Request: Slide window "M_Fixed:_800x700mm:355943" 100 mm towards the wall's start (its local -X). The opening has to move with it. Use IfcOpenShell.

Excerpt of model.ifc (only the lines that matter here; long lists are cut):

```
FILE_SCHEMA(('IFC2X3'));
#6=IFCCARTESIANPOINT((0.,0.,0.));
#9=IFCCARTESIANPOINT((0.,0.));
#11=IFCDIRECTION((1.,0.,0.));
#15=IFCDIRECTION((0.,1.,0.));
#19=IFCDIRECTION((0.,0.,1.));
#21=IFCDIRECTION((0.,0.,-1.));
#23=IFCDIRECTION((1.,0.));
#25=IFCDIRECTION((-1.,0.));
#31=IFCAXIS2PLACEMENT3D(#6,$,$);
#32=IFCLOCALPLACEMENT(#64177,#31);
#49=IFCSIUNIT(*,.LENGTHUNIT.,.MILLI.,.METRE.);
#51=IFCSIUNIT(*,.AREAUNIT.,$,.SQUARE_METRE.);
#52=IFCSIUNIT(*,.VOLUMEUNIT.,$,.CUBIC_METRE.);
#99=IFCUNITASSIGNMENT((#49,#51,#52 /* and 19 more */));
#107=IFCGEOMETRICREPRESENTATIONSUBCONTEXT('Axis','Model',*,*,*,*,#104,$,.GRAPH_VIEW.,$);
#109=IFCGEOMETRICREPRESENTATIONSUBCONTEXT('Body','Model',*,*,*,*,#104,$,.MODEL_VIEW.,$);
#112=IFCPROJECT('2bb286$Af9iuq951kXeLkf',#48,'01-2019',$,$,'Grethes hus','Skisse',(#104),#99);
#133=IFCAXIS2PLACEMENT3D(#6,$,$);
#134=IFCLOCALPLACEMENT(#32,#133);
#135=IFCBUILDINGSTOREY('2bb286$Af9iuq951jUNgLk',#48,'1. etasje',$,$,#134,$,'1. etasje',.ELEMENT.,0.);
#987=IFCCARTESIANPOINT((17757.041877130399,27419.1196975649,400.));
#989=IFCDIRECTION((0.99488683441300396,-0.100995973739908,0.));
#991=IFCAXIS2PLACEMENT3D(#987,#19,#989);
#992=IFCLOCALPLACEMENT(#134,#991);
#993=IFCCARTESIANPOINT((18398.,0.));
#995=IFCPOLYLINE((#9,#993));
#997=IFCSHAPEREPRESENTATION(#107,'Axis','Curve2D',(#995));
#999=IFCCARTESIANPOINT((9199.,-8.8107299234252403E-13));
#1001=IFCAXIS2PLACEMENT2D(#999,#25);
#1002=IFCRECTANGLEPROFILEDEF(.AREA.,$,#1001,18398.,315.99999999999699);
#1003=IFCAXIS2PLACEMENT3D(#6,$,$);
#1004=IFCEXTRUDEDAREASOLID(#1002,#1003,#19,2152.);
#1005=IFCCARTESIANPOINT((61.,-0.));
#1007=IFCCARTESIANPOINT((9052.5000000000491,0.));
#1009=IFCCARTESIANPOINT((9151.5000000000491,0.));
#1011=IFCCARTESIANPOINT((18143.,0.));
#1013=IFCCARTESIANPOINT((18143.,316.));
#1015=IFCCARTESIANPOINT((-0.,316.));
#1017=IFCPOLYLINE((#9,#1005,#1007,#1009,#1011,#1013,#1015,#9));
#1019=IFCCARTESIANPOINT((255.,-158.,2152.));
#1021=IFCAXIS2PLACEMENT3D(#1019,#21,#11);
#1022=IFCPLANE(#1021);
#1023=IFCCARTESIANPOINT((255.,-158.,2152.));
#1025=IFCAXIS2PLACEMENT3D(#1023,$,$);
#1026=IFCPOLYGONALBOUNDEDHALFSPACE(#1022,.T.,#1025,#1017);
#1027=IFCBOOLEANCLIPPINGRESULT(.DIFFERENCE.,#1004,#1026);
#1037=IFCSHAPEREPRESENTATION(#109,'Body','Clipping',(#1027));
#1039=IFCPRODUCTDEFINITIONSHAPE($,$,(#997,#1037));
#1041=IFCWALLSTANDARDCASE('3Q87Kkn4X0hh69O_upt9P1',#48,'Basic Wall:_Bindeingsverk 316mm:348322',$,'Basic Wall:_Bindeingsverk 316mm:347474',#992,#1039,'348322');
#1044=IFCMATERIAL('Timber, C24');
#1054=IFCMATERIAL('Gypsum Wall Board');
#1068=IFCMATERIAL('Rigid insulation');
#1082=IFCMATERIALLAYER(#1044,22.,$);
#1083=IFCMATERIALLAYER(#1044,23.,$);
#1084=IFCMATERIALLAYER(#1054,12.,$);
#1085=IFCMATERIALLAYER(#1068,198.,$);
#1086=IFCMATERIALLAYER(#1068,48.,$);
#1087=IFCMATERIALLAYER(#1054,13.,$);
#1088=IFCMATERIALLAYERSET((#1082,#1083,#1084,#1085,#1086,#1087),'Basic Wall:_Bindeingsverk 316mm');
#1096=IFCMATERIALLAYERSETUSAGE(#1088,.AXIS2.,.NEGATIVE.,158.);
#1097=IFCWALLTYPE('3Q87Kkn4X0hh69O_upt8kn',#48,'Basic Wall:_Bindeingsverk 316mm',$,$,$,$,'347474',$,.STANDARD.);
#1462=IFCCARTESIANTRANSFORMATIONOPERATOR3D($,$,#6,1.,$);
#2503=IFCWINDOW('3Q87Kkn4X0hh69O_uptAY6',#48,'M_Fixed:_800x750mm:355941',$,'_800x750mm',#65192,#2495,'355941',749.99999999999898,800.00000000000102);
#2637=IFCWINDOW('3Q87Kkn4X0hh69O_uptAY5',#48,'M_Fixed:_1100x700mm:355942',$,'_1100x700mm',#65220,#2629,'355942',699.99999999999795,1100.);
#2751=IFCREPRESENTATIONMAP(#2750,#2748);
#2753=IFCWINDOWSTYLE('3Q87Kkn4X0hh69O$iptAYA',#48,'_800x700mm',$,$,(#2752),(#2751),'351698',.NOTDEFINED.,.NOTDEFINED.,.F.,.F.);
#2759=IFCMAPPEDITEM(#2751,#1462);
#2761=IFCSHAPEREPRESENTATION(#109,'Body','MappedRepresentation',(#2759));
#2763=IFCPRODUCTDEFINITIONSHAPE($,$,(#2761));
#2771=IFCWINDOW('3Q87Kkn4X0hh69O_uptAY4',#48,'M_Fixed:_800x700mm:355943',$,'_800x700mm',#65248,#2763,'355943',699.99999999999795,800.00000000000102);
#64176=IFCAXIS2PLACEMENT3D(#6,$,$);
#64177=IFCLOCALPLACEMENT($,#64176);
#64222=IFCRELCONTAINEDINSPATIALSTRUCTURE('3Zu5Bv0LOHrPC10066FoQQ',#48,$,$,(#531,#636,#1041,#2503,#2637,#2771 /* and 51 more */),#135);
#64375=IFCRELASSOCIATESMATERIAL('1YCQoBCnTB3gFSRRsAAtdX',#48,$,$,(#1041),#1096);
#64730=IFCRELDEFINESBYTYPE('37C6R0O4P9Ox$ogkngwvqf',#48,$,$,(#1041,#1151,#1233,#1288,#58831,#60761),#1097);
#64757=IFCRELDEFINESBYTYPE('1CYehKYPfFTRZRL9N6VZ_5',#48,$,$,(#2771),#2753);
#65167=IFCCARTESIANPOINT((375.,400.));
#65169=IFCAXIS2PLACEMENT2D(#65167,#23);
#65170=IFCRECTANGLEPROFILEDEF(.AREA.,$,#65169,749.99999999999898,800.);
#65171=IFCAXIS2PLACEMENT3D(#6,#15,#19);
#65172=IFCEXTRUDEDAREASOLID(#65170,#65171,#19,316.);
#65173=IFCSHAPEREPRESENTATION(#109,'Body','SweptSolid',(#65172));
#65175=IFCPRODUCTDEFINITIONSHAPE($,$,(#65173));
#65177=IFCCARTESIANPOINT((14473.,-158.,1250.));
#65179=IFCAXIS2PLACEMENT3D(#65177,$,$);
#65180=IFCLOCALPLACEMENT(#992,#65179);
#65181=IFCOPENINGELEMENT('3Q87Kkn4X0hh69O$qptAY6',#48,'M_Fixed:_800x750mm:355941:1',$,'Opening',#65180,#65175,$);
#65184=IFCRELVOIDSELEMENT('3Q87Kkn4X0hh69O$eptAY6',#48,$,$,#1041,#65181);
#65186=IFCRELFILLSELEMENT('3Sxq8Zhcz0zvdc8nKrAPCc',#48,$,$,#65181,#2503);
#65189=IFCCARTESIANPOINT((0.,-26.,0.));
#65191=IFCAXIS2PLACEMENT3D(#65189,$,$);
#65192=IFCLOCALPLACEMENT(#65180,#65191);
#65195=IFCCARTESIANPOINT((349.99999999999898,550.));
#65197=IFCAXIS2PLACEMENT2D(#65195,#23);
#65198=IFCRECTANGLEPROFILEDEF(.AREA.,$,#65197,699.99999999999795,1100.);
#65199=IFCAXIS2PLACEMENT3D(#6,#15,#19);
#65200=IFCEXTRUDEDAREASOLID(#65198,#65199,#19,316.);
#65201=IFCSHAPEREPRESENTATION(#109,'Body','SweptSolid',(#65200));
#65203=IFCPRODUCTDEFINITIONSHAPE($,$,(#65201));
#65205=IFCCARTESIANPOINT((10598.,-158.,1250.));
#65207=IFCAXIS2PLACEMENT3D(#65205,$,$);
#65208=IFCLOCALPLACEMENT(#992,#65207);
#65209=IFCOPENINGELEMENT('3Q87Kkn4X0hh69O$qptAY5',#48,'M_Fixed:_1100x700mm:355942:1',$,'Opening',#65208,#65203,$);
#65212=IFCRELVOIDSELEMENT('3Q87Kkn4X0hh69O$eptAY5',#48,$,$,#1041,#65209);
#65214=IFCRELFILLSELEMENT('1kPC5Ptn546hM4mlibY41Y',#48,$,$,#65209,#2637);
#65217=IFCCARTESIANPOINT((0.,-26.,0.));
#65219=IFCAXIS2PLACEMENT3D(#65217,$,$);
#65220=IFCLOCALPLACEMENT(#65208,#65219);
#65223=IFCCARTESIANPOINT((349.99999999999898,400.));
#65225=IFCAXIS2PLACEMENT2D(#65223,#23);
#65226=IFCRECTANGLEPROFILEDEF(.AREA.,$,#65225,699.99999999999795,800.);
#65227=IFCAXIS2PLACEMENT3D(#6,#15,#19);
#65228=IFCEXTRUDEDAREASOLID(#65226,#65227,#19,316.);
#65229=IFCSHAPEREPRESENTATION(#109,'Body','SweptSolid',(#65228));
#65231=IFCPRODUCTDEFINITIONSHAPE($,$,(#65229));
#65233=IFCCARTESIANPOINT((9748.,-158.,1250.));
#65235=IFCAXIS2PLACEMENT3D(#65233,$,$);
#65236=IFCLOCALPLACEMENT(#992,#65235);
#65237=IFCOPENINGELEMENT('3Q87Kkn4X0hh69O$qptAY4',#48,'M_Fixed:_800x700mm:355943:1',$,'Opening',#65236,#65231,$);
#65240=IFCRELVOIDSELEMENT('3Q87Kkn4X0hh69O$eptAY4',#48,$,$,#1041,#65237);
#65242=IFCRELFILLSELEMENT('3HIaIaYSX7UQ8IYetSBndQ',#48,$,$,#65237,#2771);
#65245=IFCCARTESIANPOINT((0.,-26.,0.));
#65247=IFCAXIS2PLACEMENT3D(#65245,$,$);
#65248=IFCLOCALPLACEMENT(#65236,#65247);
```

```python
import ifcopenshell
import ifcopenshell.api.geometry
import ifcopenshell.util.placement
import ifcopenshell.util.unit

model = ifcopenshell.open("model.ifc")
unit_scale = ifcopenshell.util.unit.calculate_unit_scale(model)

window = model.by_guid("3Q87Kkn4X0hh69O_uptAY4")
opening = window.FillsVoids[0].RelatingOpeningElement
wall = opening.VoidsElements[0].RelatingBuildingElement

wall_matrix = ifcopenshell.util.placement.get_local_placement(wall.ObjectPlacement)
shift = wall_matrix[:3, 0] * -0.1 / unit_scale
before = ifcopenshell.util.placement.get_local_placement(window.ObjectPlacement)[:3, 3].copy()

# The window is placed relative to its opening, so it follows when the opening moves.
matrix = ifcopenshell.util.placement.get_local_placement(opening.ObjectPlacement)
matrix[:3, 3] += shift
ifcopenshell.api.geometry.edit_object_placement(
    model, product=opening, matrix=matrix, is_si=False, should_transform_children=True
)

after = ifcopenshell.util.placement.get_local_placement(window.ObjectPlacement)[:3, 3]
print("window moved by", (after - before).round(3) + 0.0)

model.write("model_edited.ifc")
```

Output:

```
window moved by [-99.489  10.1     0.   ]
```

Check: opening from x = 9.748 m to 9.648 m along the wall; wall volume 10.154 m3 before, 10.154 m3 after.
